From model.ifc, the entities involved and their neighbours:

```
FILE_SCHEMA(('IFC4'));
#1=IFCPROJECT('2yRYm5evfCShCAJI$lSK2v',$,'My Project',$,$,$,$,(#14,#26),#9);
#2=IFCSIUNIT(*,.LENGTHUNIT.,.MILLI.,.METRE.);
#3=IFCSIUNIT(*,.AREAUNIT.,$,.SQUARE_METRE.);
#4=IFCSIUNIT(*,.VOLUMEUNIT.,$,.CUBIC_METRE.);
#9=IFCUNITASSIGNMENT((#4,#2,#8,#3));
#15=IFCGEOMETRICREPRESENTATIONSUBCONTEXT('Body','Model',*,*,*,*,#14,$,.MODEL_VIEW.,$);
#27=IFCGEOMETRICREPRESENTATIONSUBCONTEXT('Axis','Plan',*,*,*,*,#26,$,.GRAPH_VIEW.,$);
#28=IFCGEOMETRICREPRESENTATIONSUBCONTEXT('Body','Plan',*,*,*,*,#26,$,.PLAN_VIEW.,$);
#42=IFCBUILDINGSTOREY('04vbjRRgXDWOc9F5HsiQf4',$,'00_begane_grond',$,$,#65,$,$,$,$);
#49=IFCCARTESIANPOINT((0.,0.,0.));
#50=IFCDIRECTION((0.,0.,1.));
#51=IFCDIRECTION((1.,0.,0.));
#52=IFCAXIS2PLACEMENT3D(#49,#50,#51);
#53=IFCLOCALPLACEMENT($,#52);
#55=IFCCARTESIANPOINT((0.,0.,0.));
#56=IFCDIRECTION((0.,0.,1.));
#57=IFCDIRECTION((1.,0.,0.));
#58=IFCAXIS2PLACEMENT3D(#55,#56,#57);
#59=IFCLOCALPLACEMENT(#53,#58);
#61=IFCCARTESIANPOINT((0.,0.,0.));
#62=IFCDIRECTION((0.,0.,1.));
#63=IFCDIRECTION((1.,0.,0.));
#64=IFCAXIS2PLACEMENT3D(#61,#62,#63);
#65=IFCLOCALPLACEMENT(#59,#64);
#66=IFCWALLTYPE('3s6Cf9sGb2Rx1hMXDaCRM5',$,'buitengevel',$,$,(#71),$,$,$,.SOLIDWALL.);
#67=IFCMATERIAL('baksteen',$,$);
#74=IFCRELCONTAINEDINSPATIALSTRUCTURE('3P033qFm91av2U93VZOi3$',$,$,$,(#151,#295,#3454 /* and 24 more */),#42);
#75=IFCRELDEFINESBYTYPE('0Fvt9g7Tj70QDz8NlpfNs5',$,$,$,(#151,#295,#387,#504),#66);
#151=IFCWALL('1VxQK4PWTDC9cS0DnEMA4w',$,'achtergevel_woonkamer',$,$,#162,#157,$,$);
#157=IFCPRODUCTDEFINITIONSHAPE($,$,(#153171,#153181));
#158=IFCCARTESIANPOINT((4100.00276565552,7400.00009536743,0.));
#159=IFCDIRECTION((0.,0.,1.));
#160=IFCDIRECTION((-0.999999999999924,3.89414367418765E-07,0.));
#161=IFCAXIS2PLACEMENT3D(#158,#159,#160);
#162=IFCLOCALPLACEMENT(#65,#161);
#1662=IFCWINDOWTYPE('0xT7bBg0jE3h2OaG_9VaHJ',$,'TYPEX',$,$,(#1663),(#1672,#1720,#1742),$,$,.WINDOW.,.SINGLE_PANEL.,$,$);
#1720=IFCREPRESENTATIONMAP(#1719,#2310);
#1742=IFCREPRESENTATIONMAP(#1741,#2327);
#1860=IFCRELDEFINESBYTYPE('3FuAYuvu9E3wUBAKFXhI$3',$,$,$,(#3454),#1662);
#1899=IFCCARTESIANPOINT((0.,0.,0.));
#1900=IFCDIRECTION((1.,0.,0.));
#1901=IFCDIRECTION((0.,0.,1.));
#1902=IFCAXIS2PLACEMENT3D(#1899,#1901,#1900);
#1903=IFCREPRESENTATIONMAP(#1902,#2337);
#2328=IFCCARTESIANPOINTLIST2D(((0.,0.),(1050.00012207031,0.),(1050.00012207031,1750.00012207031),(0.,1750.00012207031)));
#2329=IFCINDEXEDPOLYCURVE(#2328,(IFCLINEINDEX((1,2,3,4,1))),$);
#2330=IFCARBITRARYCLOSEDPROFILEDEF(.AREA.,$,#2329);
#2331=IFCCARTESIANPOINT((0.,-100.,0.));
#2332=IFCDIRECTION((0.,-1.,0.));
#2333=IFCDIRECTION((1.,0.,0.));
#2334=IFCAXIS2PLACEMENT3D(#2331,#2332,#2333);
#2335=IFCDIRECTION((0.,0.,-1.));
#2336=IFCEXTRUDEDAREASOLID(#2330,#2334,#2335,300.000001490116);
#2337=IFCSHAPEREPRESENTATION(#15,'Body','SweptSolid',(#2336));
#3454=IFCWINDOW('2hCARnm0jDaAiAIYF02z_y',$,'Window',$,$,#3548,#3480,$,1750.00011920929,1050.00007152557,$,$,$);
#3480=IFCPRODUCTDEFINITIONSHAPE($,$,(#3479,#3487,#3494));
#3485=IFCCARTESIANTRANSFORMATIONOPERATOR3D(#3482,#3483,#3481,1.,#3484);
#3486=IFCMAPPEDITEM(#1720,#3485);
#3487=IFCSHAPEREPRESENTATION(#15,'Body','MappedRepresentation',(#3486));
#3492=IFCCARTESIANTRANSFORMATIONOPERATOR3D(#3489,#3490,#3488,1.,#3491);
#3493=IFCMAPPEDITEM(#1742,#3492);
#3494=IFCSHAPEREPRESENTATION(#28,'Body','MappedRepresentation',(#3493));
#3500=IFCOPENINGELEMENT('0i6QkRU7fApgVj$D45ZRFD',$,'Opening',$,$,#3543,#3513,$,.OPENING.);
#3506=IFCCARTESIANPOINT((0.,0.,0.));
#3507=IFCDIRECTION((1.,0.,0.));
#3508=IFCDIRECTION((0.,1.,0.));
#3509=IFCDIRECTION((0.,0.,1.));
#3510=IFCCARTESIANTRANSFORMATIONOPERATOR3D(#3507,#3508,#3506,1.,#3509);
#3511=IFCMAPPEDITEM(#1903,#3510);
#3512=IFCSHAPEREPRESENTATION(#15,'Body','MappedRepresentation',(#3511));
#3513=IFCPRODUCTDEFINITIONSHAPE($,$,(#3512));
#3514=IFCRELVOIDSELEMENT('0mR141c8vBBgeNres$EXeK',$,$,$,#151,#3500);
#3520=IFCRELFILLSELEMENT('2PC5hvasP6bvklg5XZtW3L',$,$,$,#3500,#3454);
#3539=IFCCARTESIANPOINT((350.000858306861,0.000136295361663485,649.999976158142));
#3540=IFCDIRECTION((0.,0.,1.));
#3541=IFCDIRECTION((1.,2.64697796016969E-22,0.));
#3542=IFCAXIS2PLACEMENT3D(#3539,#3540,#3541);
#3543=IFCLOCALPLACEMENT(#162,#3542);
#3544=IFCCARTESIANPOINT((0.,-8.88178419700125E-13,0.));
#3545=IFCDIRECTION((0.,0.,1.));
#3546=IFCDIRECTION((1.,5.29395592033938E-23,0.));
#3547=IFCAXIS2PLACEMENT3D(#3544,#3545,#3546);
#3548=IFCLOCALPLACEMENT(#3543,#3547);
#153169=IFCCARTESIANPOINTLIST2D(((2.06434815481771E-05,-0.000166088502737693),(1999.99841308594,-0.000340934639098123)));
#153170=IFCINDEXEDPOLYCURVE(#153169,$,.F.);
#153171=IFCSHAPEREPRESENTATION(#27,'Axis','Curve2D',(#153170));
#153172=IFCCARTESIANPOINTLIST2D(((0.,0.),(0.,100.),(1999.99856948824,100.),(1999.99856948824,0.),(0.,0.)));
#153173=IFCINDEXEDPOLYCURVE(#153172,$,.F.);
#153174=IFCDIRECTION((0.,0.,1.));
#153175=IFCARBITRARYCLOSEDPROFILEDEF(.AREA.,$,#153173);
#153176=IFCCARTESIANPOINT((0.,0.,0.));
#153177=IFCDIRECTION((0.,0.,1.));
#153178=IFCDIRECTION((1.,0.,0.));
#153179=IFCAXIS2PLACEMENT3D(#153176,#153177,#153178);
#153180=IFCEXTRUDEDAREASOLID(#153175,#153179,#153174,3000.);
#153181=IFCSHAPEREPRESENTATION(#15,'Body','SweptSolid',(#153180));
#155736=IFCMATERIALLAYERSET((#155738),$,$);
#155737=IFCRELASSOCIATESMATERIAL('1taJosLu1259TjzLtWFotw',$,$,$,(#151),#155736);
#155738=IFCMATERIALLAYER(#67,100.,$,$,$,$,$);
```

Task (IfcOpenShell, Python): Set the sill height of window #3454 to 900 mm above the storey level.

```python
import numpy as np
import ifcopenshell
import ifcopenshell.api.geometry
import ifcopenshell.geom
import ifcopenshell.util.element
import ifcopenshell.util.placement
import ifcopenshell.util.shape
import ifcopenshell.util.unit

model = ifcopenshell.open("model.ifc")
unit_scale = ifcopenshell.util.unit.calculate_unit_scale(model)

window = model.by_id(3454)
opening = window.FillsVoids[0].RelatingOpeningElement
storey = ifcopenshell.util.element.get_container(window, ifc_class="IfcBuildingStorey")
level = ifcopenshell.util.placement.get_local_placement(storey.ObjectPlacement)[2, 3]

# The opening's origin need not be at the sill, so measure its lowest point.
shape = ifcopenshell.geom.create_shape(ifcopenshell.geom.settings(), opening)
bottom = ifcopenshell.util.shape.get_shape_bottom_elevation(shape, shape.geometry) / unit_scale
dz = level + 900.0 - bottom

shift = np.array([0.0, 0.0, dz])
# The window is placed relative to its opening, so it follows when the opening moves.
matrix = ifcopenshell.util.placement.get_local_placement(opening.ObjectPlacement)
matrix[:3, 3] += shift
ifcopenshell.api.geometry.edit_object_placement(
    model, product=opening, matrix=matrix, is_si=False, should_transform_children=True
)

print(f"moved by {dz * unit_scale:+.3f} m")

model.write("model_rev.ifc")
```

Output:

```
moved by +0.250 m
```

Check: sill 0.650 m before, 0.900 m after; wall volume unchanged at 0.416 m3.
